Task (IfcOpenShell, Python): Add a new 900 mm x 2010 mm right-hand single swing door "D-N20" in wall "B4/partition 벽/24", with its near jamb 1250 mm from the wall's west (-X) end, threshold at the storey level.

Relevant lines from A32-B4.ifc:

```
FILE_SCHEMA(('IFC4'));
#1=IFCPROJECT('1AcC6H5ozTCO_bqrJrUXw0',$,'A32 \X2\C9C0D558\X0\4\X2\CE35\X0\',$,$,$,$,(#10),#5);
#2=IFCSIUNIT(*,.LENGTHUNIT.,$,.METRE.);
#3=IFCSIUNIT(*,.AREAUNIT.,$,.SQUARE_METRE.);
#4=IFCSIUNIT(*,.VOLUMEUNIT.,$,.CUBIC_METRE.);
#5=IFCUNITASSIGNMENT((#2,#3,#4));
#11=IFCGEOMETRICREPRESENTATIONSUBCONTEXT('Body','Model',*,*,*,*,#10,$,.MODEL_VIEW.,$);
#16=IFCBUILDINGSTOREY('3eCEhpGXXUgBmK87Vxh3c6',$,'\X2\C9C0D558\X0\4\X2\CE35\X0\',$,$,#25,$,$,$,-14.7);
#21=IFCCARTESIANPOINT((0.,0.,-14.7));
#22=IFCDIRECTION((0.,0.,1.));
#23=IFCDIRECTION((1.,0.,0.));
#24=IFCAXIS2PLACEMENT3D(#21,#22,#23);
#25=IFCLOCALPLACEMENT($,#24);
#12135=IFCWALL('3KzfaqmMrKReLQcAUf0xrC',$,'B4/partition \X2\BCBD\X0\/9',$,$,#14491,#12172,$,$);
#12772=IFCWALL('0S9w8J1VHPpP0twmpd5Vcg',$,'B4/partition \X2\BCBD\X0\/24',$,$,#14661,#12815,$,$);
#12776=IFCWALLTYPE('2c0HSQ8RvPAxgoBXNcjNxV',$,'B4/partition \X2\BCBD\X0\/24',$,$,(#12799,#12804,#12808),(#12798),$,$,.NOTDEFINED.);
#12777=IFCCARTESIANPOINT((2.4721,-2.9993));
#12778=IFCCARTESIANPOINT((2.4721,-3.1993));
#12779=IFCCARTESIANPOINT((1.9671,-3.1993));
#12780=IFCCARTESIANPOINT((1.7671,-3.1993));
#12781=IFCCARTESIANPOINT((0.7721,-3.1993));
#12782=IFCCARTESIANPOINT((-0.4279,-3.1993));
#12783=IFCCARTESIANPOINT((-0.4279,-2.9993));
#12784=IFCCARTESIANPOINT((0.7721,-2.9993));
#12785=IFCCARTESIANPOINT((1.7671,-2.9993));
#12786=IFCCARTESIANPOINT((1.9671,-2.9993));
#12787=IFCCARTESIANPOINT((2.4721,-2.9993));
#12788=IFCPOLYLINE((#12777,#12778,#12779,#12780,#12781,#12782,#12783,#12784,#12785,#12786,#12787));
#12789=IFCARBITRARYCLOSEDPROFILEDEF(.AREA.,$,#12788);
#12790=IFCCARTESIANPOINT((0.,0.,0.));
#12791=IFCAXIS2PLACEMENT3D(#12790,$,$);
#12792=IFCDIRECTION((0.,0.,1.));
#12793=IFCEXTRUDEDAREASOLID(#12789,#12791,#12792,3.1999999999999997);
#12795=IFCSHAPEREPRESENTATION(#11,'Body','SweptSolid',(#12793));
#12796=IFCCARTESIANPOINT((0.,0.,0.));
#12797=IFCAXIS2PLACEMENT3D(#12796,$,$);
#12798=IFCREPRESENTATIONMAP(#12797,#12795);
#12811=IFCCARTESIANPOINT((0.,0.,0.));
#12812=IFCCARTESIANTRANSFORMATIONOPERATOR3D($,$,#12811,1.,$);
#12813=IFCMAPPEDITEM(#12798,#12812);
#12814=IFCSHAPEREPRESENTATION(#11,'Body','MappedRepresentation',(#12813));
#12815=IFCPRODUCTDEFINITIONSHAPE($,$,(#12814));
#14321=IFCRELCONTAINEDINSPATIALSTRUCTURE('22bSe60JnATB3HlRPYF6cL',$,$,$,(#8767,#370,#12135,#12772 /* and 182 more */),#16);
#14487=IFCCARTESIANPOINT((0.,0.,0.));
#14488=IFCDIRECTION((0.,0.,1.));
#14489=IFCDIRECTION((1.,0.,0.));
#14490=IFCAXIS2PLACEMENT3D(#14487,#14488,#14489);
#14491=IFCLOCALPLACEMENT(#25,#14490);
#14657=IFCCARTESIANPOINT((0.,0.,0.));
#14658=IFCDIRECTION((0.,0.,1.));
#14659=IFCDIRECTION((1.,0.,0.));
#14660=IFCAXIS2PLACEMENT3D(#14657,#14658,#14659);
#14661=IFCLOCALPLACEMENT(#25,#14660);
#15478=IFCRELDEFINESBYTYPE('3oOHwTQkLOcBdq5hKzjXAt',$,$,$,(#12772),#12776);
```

```python
import numpy as np
import ifcopenshell
import ifcopenshell.api.feature
import ifcopenshell.api.geometry
import ifcopenshell.api.root
import ifcopenshell.api.spatial
import ifcopenshell.geom
import ifcopenshell.util.element
import ifcopenshell.util.placement
import ifcopenshell.util.representation
import ifcopenshell.util.shape
import ifcopenshell.util.unit

model = ifcopenshell.open("A32-B4.ifc")
unit_scale = ifcopenshell.util.unit.calculate_unit_scale(model)
settings = ifcopenshell.geom.settings()


def volume(element):
    """Net volume in cubic metres, openings subtracted."""
    shape = ifcopenshell.geom.create_shape(settings, element)
    return ifcopenshell.util.shape.get_volume(shape.geometry)


wall = model.by_guid("0S9w8J1VHPpP0twmpd5Vcg")
storey = ifcopenshell.util.element.get_container(wall, ifc_class="IfcBuildingStorey")
context = ifcopenshell.util.representation.get_context(model, "Model", "Body", "MODEL_VIEW")
before = volume(wall)

width, height, from_end, sill = 0.9, 2.01, 1.25, 0.0  # metres

# The wall runs along its own X axis, and the end named is its -X end.
wall_shape = ifcopenshell.geom.create_shape(settings, wall)
x, y, z = ifcopenshell.util.shape.get_vertices(wall_shape.geometry).T
start = x.min() + from_end
face, thickness = float(y.min()), float(y.max() - y.min())
wall_matrix = ifcopenshell.util.placement.get_local_placement(wall.ObjectPlacement)
level = ifcopenshell.util.placement.get_local_placement(storey.ObjectPlacement)[2, 3]


def in_wall(x, y):
    """Placement at x, y metres in the wall's axes, at sill height."""
    matrix = wall_matrix.copy()
    matrix[:, 3] = wall_matrix @ np.array([x / unit_scale, y / unit_scale, 0.0, 1.0])
    matrix[2, 3] = level + sill / unit_scale
    return matrix


# Opening: a box that overshoots both wall faces by 50 mm.
opening = ifcopenshell.api.root.create_entity(model, ifc_class="IfcOpeningElement", predefined_type="OPENING")
box = ifcopenshell.api.geometry.add_wall_representation(
    model, context=context, length=width, height=height, thickness=thickness + 0.1
)
ifcopenshell.api.geometry.assign_representation(model, product=opening, representation=box)
ifcopenshell.api.geometry.edit_object_placement(model, product=opening, matrix=in_wall(start, face - 0.05), is_si=False)
ifcopenshell.api.feature.add_feature(model, feature=opening, element=wall)

door = ifcopenshell.api.root.create_entity(model, ifc_class="IfcDoor", name="D-N20", predefined_type="DOOR")
door.OverallWidth, door.OverallHeight = width / unit_scale, height / unit_scale
door.OperationType = "SINGLE_SWING_RIGHT"
body = ifcopenshell.api.geometry.add_door_representation(
    model,
    context=context,
    overall_width=door.OverallWidth,
    overall_height=door.OverallHeight,
    operation_type="SINGLE_SWING_RIGHT",
    lining_properties={"LiningDepth": thickness / unit_scale, "ThresholdDepth": thickness / unit_scale},
)
ifcopenshell.api.geometry.assign_representation(model, product=door, representation=body)
ifcopenshell.api.spatial.assign_container(model, products=[door], relating_structure=storey)
ifcopenshell.api.feature.add_filling(model, opening=opening, element=door)

# The lining spans the wall, so the door starts at the wall face.
ifcopenshell.api.geometry.edit_object_placement(model, product=door, matrix=in_wall(start, face), is_si=False)

after = volume(wall)

print(f"wall volume {before:.3f} -> {after:.3f} m3")

model.write("A32-B4_updated.ifc")
```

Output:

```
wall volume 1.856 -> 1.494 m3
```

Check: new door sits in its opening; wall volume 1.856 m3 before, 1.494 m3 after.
